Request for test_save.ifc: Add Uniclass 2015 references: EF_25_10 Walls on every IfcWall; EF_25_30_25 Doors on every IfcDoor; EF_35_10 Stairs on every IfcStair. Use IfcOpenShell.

First a look at what the model holds.

```python
import ifcopenshell

model = ifcopenshell.open("test_save.ifc")
print(model.schema)
print("classifications:", [c.Name for c in model.by_type("IfcClassification")])
for ifc_class in ("IfcDoor", "IfcRoof", "IfcStair", "IfcWall", "IfcWindow"):
    print(ifc_class, len(model.by_type(ifc_class)))
```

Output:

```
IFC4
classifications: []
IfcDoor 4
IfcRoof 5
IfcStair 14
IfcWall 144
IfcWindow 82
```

```python
import ifcopenshell
import ifcopenshell.api.classification

model = ifcopenshell.open("test_save.ifc")

system = ifcopenshell.api.classification.add_classification(model, classification="Uniclass 2015")

codes = {
    "IfcWall": ("EF_25_10", "Walls"),
    "IfcDoor": ("EF_25_30_25", "Doors"),
    "IfcStair": ("EF_35_10", "Stairs"),
}
for ifc_class, (code, name) in codes.items():
    products = model.by_type(ifc_class)
    ifcopenshell.api.classification.add_reference(
        model, products=products, classification=system, identification=code, name=name
    )
    print(code, len(products))

model.write("test_save_updated.ifc")
```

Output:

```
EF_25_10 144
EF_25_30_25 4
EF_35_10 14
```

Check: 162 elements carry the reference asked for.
